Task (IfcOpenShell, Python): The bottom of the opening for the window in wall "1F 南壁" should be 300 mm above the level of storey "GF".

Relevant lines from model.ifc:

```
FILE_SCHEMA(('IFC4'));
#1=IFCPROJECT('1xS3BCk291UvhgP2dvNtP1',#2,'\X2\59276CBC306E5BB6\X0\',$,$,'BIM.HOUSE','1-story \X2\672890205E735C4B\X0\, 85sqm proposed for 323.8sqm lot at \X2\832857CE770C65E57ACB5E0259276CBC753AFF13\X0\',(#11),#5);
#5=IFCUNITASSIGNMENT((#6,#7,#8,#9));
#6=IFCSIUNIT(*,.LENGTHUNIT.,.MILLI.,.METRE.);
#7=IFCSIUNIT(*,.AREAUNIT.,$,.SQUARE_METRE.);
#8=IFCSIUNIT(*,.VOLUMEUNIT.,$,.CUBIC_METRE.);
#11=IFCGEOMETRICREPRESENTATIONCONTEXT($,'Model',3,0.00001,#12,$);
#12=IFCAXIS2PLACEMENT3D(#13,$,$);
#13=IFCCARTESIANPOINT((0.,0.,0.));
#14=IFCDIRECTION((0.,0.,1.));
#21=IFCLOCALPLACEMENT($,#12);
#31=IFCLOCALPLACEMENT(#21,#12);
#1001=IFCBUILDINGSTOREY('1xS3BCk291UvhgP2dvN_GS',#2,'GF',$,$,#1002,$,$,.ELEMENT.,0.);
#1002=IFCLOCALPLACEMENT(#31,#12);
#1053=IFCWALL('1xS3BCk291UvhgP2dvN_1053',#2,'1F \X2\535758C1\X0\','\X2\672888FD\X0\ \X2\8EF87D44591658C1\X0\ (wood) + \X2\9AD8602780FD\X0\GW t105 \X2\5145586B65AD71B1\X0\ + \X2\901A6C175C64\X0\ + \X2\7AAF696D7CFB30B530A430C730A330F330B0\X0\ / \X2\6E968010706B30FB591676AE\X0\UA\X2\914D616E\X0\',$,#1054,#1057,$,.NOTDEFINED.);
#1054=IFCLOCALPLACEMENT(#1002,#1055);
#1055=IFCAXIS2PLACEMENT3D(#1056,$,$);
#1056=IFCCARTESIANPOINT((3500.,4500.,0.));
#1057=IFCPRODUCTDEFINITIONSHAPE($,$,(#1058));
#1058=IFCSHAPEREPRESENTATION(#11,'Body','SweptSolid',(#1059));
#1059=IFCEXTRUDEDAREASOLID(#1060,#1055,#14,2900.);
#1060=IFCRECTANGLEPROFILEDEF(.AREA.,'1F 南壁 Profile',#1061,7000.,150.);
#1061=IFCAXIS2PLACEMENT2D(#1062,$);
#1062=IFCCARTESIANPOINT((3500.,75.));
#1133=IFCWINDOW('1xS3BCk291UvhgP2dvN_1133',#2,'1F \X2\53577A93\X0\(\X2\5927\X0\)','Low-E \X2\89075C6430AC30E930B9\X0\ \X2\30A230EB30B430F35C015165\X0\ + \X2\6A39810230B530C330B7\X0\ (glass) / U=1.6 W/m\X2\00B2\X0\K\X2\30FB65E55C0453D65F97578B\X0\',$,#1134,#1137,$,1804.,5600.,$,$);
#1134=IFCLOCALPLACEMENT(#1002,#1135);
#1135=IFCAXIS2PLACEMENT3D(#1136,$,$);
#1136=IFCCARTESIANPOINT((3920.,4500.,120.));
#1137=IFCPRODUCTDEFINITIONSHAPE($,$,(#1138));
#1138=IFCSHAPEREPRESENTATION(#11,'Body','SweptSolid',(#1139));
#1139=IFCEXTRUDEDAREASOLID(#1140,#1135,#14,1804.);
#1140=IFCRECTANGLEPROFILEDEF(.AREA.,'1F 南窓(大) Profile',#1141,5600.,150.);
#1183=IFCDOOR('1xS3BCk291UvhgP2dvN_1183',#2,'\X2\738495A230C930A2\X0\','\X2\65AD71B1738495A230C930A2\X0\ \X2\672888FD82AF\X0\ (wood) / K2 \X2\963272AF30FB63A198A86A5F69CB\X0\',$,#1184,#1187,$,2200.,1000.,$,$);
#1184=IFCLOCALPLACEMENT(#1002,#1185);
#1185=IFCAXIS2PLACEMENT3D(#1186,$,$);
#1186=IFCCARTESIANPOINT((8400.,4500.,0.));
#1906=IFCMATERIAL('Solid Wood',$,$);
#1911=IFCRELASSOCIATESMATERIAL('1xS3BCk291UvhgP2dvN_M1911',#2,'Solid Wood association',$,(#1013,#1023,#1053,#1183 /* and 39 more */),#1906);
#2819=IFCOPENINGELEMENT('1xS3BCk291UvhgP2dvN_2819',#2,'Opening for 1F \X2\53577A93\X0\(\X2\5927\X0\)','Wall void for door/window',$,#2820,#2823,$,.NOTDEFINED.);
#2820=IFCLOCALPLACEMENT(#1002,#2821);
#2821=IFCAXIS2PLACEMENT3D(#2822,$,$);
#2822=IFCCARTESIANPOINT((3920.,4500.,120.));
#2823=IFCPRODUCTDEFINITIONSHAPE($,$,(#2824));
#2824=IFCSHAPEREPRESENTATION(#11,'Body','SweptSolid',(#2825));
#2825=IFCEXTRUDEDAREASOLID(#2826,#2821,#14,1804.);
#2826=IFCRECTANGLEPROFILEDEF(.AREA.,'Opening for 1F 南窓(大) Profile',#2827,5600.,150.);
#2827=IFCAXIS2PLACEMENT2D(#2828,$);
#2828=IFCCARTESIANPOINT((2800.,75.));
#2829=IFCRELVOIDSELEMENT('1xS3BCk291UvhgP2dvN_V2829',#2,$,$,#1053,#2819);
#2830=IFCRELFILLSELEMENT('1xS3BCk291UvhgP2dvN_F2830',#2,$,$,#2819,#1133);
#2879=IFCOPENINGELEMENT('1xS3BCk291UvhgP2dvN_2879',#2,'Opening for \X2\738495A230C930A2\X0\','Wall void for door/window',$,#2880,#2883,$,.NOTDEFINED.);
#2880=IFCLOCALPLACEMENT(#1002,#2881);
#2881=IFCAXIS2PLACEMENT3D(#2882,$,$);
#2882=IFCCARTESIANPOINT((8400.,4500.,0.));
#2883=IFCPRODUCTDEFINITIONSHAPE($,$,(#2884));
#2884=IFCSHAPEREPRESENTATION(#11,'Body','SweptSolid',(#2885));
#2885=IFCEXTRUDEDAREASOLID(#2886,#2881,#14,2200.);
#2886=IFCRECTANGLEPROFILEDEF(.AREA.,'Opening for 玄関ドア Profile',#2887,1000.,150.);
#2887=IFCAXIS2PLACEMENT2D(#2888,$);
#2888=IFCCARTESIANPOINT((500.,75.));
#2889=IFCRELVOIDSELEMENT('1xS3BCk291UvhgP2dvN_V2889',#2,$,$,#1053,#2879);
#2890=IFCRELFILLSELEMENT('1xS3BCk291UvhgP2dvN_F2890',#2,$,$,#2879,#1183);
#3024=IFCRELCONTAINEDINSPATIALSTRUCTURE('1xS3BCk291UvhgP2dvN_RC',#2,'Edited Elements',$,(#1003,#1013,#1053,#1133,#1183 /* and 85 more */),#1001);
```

```python
import numpy as np
import ifcopenshell
import ifcopenshell.api.geometry
import ifcopenshell.geom
import ifcopenshell.util.element
import ifcopenshell.util.placement
import ifcopenshell.util.shape
import ifcopenshell.util.unit

model = ifcopenshell.open("model.ifc")
unit_scale = ifcopenshell.util.unit.calculate_unit_scale(model)

window = model.by_guid("1xS3BCk291UvhgP2dvN_1133")
opening = window.FillsVoids[0].RelatingOpeningElement
storey = ifcopenshell.util.element.get_container(window, ifc_class="IfcBuildingStorey")
level = ifcopenshell.util.placement.get_local_placement(storey.ObjectPlacement)[2, 3]

# The opening's origin need not be at the sill, so measure its lowest point.
shape = ifcopenshell.geom.create_shape(ifcopenshell.geom.settings(), opening)
bottom = ifcopenshell.util.shape.get_shape_bottom_elevation(shape, shape.geometry) / unit_scale
dz = level + 300.0 - bottom

shift = np.array([0.0, 0.0, dz])
# The window is not placed relative to its opening, so move both.
for product in (opening, window):
    matrix = ifcopenshell.util.placement.get_local_placement(product.ObjectPlacement)
    matrix[:3, 3] += shift
    ifcopenshell.api.geometry.edit_object_placement(model, product=product, matrix=matrix, is_si=False)

print(f"moved by {dz * unit_scale:+.3f} m")

model.write("model_rev.ifc")
```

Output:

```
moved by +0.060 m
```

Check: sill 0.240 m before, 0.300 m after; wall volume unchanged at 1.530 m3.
